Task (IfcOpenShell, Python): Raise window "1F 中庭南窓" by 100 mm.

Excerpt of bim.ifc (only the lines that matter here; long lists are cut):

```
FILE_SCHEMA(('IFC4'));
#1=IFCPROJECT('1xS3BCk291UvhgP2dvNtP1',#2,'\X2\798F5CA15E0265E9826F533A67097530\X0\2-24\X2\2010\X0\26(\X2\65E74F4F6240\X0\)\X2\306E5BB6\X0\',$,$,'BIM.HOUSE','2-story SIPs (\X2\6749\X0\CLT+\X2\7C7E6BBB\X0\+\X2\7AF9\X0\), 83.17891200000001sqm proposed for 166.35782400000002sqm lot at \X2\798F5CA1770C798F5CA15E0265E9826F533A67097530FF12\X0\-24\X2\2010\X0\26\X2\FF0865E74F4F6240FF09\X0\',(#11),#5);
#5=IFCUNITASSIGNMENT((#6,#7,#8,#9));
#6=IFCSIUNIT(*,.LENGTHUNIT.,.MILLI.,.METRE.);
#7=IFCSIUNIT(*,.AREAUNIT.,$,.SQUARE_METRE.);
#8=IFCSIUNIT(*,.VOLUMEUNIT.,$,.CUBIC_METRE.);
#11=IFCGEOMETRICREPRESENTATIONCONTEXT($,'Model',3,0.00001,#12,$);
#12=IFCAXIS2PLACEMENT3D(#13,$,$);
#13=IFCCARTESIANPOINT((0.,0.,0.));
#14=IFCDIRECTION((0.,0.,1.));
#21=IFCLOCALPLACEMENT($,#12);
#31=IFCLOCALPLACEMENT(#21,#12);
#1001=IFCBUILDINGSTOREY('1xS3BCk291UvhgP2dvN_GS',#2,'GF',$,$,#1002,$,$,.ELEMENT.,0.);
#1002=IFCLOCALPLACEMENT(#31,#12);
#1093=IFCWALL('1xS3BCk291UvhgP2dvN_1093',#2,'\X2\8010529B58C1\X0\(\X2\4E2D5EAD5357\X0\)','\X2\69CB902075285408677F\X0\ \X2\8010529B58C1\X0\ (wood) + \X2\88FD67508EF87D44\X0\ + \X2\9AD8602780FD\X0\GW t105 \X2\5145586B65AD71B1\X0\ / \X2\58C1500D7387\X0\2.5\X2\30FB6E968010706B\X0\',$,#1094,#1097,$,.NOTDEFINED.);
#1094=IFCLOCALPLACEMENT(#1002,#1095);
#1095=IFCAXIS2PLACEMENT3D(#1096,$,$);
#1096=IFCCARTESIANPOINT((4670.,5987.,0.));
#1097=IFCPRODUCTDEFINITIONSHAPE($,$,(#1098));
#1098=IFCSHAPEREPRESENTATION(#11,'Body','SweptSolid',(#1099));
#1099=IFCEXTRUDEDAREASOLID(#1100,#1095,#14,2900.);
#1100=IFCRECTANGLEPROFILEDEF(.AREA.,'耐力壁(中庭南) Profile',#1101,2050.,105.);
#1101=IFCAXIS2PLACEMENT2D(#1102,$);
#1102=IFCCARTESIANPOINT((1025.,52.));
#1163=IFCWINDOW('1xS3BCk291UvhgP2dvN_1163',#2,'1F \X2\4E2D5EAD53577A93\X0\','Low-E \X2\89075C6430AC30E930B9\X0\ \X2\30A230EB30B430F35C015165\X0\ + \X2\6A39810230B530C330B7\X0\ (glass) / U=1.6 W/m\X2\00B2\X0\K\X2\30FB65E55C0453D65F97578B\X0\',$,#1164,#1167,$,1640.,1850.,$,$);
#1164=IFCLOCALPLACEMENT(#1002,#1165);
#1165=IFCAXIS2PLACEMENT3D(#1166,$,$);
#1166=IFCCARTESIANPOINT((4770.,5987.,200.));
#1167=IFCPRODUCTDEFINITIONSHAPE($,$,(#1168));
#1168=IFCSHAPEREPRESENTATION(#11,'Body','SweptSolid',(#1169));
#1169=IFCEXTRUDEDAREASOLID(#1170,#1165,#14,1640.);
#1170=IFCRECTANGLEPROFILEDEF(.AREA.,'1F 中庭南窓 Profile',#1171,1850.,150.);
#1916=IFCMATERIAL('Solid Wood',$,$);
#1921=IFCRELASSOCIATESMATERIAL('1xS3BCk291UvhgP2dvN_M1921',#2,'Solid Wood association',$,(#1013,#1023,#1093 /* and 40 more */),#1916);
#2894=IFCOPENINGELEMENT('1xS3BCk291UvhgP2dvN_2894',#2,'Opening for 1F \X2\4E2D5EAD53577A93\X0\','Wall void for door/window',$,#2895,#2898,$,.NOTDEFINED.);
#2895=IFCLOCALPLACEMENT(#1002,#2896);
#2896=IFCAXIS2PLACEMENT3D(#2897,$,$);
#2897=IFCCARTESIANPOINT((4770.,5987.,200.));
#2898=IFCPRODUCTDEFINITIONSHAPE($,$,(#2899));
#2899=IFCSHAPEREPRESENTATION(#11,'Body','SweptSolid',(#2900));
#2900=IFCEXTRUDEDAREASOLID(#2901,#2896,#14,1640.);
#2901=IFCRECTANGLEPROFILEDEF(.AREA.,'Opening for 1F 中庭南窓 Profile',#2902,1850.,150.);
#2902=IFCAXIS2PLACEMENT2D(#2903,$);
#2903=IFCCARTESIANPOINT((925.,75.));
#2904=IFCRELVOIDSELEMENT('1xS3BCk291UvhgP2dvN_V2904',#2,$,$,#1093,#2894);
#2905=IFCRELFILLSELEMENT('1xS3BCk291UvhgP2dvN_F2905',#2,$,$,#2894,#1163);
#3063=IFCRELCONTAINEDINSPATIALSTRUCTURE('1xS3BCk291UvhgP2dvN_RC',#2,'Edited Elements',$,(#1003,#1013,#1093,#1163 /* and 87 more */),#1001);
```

```python
import numpy as np
import ifcopenshell
import ifcopenshell.api.geometry
import ifcopenshell.util.placement
import ifcopenshell.util.unit

model = ifcopenshell.open("bim.ifc")
unit_scale = ifcopenshell.util.unit.calculate_unit_scale(model)

window = model.by_guid("1xS3BCk291UvhgP2dvN_1163")
opening = window.FillsVoids[0].RelatingOpeningElement
dz = 100.0

shift = np.array([0.0, 0.0, dz])
# The window is not placed relative to its opening, so move both.
for product in (opening, window):
    matrix = ifcopenshell.util.placement.get_local_placement(product.ObjectPlacement)
    matrix[:3, 3] += shift
    ifcopenshell.api.geometry.edit_object_placement(model, product=product, matrix=matrix, is_si=False)

print(f"moved by {dz * unit_scale:+.3f} m")

model.write("bim_rev.ifc")
```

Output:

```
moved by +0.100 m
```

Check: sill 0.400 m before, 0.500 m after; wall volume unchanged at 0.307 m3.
